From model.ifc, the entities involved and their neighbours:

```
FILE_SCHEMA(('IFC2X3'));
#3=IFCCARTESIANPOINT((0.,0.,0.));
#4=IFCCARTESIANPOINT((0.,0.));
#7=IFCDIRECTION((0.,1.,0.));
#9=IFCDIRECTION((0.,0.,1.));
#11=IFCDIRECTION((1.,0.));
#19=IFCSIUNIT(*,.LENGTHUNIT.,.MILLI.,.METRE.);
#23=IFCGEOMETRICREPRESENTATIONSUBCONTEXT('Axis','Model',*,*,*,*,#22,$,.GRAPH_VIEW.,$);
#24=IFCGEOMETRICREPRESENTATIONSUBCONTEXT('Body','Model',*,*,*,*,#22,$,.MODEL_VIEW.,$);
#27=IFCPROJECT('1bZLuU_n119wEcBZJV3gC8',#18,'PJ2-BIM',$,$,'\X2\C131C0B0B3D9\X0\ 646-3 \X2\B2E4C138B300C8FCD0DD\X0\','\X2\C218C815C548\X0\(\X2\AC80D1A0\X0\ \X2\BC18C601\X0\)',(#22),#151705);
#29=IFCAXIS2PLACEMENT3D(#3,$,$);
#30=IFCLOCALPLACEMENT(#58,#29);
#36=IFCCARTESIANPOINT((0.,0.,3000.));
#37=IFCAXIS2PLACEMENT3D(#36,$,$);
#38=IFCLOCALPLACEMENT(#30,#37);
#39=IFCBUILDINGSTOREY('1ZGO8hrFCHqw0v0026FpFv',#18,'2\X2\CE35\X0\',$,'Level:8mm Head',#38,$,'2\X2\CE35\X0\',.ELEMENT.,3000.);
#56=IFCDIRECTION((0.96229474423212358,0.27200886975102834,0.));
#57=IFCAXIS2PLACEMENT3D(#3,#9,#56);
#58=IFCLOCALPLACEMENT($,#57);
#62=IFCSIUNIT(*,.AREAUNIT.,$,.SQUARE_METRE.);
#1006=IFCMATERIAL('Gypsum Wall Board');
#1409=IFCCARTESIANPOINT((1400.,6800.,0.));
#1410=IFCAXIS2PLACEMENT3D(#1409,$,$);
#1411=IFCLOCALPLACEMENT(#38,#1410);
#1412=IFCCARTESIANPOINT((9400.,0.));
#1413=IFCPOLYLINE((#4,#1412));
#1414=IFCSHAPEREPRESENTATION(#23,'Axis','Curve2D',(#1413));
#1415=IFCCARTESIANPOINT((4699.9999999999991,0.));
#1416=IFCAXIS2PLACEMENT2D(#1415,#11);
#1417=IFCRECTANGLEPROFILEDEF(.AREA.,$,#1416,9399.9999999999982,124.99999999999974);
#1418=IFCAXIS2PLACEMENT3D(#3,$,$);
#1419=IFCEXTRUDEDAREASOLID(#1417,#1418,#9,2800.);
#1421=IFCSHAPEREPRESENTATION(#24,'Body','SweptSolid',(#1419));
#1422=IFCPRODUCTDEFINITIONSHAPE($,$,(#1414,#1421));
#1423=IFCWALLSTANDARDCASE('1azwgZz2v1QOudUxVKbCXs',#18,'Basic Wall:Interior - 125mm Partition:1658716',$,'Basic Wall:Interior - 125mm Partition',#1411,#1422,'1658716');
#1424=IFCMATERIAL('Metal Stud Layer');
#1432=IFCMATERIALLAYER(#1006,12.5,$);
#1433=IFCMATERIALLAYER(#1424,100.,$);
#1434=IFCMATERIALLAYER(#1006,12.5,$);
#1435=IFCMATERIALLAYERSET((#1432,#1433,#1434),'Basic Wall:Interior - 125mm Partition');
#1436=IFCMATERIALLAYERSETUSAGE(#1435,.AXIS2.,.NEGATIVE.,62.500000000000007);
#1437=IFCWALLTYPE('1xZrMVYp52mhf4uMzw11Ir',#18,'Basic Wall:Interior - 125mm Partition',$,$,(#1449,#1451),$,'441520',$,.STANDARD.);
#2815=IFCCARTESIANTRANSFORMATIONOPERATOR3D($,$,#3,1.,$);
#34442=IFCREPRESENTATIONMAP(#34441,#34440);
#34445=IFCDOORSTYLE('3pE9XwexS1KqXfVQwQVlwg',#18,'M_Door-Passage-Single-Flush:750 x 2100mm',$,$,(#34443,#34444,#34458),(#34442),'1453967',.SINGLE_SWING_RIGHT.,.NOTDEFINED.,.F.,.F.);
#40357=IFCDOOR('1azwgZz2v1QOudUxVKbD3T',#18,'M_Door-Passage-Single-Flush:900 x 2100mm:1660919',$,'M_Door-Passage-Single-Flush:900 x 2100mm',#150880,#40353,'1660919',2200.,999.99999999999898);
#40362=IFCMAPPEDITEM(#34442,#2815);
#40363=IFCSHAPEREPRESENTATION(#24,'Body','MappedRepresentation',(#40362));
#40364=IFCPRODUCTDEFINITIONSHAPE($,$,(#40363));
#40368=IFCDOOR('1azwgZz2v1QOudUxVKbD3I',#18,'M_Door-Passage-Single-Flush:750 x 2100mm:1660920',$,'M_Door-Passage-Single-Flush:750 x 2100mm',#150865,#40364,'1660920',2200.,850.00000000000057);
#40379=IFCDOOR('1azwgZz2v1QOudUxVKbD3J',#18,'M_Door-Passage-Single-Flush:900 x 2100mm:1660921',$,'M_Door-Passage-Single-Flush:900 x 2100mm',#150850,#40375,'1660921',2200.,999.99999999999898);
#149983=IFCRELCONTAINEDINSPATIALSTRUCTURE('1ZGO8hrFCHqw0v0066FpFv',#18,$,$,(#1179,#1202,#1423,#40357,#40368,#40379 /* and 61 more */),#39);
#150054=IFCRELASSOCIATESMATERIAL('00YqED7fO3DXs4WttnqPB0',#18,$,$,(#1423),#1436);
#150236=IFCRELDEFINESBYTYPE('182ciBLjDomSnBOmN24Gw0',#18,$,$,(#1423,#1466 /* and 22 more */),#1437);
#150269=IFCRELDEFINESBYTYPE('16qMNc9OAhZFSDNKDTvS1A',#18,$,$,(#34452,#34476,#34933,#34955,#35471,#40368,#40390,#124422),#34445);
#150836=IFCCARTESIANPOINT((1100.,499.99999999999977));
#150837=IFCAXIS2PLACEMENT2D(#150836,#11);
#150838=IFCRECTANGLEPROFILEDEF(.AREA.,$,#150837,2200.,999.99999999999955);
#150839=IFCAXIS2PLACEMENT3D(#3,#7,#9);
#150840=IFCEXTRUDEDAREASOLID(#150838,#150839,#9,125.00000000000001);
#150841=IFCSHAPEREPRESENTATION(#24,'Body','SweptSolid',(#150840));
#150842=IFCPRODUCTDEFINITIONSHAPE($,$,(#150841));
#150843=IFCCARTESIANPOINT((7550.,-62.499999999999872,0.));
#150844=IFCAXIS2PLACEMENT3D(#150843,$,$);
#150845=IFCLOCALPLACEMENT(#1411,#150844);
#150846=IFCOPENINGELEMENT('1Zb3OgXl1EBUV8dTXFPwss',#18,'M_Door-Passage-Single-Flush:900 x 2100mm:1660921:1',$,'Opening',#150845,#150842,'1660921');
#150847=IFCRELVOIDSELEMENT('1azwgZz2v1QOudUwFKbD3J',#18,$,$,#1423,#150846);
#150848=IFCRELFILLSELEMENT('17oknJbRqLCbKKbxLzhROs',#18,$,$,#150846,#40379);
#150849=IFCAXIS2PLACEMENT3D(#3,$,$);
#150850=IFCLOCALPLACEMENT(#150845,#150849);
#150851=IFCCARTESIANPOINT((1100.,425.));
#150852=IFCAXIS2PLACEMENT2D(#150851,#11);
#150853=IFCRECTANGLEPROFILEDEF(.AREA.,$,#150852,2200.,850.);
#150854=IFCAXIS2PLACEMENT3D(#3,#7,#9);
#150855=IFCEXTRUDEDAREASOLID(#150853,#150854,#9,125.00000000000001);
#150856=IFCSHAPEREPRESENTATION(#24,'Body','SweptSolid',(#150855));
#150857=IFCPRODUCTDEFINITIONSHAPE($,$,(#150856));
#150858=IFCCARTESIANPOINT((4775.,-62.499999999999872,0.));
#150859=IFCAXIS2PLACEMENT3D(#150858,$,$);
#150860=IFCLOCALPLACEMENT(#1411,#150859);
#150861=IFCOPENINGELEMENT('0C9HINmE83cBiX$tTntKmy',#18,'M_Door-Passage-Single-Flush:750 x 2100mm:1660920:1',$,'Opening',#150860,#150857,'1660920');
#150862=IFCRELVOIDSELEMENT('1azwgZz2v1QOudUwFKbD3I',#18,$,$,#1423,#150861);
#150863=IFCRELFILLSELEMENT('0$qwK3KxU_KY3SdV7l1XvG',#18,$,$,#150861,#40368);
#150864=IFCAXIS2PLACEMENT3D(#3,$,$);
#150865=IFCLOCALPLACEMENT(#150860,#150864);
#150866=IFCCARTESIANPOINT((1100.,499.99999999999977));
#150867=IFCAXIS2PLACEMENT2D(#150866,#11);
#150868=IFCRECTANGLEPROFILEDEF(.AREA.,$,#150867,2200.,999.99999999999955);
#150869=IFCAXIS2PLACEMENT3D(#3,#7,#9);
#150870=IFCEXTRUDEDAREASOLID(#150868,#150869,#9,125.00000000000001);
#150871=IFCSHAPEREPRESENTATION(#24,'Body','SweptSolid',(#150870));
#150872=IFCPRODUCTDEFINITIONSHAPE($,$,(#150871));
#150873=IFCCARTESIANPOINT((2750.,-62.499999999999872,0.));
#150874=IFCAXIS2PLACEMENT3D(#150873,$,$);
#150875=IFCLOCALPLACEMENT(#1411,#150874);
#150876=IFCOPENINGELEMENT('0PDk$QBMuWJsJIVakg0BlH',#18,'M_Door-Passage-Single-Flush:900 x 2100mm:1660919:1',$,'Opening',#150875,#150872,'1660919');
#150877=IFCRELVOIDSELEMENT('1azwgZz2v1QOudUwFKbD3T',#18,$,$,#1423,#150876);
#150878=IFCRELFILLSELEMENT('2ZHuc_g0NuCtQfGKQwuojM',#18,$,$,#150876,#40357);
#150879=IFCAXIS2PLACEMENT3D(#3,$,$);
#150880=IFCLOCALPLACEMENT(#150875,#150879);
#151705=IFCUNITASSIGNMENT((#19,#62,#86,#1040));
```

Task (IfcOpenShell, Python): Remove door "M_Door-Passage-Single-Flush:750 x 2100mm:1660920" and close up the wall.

```python
import ifcopenshell
import ifcopenshell.api.feature
import ifcopenshell.api.root
import ifcopenshell.geom
import ifcopenshell.util.shape

model = ifcopenshell.open("model.ifc")
settings = ifcopenshell.geom.settings()


def volume(element):
    """Net volume in cubic metres, openings subtracted."""
    shape = ifcopenshell.geom.create_shape(settings, element)
    return ifcopenshell.util.shape.get_volume(shape.geometry)


door = model.by_id(40368)
opening = door.FillsVoids[0].RelatingOpeningElement
wall = opening.VoidsElements[0].RelatingBuildingElement
before = volume(wall)

ifcopenshell.api.root.remove_product(model, product=door)
ifcopenshell.api.feature.remove_feature(model, feature=opening)

after = volume(wall)

print(f"wall volume {before:.3f} -> {after:.3f} m3")

model.write("model_edited.ifc")
```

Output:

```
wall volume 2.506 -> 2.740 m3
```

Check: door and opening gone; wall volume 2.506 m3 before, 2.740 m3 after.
